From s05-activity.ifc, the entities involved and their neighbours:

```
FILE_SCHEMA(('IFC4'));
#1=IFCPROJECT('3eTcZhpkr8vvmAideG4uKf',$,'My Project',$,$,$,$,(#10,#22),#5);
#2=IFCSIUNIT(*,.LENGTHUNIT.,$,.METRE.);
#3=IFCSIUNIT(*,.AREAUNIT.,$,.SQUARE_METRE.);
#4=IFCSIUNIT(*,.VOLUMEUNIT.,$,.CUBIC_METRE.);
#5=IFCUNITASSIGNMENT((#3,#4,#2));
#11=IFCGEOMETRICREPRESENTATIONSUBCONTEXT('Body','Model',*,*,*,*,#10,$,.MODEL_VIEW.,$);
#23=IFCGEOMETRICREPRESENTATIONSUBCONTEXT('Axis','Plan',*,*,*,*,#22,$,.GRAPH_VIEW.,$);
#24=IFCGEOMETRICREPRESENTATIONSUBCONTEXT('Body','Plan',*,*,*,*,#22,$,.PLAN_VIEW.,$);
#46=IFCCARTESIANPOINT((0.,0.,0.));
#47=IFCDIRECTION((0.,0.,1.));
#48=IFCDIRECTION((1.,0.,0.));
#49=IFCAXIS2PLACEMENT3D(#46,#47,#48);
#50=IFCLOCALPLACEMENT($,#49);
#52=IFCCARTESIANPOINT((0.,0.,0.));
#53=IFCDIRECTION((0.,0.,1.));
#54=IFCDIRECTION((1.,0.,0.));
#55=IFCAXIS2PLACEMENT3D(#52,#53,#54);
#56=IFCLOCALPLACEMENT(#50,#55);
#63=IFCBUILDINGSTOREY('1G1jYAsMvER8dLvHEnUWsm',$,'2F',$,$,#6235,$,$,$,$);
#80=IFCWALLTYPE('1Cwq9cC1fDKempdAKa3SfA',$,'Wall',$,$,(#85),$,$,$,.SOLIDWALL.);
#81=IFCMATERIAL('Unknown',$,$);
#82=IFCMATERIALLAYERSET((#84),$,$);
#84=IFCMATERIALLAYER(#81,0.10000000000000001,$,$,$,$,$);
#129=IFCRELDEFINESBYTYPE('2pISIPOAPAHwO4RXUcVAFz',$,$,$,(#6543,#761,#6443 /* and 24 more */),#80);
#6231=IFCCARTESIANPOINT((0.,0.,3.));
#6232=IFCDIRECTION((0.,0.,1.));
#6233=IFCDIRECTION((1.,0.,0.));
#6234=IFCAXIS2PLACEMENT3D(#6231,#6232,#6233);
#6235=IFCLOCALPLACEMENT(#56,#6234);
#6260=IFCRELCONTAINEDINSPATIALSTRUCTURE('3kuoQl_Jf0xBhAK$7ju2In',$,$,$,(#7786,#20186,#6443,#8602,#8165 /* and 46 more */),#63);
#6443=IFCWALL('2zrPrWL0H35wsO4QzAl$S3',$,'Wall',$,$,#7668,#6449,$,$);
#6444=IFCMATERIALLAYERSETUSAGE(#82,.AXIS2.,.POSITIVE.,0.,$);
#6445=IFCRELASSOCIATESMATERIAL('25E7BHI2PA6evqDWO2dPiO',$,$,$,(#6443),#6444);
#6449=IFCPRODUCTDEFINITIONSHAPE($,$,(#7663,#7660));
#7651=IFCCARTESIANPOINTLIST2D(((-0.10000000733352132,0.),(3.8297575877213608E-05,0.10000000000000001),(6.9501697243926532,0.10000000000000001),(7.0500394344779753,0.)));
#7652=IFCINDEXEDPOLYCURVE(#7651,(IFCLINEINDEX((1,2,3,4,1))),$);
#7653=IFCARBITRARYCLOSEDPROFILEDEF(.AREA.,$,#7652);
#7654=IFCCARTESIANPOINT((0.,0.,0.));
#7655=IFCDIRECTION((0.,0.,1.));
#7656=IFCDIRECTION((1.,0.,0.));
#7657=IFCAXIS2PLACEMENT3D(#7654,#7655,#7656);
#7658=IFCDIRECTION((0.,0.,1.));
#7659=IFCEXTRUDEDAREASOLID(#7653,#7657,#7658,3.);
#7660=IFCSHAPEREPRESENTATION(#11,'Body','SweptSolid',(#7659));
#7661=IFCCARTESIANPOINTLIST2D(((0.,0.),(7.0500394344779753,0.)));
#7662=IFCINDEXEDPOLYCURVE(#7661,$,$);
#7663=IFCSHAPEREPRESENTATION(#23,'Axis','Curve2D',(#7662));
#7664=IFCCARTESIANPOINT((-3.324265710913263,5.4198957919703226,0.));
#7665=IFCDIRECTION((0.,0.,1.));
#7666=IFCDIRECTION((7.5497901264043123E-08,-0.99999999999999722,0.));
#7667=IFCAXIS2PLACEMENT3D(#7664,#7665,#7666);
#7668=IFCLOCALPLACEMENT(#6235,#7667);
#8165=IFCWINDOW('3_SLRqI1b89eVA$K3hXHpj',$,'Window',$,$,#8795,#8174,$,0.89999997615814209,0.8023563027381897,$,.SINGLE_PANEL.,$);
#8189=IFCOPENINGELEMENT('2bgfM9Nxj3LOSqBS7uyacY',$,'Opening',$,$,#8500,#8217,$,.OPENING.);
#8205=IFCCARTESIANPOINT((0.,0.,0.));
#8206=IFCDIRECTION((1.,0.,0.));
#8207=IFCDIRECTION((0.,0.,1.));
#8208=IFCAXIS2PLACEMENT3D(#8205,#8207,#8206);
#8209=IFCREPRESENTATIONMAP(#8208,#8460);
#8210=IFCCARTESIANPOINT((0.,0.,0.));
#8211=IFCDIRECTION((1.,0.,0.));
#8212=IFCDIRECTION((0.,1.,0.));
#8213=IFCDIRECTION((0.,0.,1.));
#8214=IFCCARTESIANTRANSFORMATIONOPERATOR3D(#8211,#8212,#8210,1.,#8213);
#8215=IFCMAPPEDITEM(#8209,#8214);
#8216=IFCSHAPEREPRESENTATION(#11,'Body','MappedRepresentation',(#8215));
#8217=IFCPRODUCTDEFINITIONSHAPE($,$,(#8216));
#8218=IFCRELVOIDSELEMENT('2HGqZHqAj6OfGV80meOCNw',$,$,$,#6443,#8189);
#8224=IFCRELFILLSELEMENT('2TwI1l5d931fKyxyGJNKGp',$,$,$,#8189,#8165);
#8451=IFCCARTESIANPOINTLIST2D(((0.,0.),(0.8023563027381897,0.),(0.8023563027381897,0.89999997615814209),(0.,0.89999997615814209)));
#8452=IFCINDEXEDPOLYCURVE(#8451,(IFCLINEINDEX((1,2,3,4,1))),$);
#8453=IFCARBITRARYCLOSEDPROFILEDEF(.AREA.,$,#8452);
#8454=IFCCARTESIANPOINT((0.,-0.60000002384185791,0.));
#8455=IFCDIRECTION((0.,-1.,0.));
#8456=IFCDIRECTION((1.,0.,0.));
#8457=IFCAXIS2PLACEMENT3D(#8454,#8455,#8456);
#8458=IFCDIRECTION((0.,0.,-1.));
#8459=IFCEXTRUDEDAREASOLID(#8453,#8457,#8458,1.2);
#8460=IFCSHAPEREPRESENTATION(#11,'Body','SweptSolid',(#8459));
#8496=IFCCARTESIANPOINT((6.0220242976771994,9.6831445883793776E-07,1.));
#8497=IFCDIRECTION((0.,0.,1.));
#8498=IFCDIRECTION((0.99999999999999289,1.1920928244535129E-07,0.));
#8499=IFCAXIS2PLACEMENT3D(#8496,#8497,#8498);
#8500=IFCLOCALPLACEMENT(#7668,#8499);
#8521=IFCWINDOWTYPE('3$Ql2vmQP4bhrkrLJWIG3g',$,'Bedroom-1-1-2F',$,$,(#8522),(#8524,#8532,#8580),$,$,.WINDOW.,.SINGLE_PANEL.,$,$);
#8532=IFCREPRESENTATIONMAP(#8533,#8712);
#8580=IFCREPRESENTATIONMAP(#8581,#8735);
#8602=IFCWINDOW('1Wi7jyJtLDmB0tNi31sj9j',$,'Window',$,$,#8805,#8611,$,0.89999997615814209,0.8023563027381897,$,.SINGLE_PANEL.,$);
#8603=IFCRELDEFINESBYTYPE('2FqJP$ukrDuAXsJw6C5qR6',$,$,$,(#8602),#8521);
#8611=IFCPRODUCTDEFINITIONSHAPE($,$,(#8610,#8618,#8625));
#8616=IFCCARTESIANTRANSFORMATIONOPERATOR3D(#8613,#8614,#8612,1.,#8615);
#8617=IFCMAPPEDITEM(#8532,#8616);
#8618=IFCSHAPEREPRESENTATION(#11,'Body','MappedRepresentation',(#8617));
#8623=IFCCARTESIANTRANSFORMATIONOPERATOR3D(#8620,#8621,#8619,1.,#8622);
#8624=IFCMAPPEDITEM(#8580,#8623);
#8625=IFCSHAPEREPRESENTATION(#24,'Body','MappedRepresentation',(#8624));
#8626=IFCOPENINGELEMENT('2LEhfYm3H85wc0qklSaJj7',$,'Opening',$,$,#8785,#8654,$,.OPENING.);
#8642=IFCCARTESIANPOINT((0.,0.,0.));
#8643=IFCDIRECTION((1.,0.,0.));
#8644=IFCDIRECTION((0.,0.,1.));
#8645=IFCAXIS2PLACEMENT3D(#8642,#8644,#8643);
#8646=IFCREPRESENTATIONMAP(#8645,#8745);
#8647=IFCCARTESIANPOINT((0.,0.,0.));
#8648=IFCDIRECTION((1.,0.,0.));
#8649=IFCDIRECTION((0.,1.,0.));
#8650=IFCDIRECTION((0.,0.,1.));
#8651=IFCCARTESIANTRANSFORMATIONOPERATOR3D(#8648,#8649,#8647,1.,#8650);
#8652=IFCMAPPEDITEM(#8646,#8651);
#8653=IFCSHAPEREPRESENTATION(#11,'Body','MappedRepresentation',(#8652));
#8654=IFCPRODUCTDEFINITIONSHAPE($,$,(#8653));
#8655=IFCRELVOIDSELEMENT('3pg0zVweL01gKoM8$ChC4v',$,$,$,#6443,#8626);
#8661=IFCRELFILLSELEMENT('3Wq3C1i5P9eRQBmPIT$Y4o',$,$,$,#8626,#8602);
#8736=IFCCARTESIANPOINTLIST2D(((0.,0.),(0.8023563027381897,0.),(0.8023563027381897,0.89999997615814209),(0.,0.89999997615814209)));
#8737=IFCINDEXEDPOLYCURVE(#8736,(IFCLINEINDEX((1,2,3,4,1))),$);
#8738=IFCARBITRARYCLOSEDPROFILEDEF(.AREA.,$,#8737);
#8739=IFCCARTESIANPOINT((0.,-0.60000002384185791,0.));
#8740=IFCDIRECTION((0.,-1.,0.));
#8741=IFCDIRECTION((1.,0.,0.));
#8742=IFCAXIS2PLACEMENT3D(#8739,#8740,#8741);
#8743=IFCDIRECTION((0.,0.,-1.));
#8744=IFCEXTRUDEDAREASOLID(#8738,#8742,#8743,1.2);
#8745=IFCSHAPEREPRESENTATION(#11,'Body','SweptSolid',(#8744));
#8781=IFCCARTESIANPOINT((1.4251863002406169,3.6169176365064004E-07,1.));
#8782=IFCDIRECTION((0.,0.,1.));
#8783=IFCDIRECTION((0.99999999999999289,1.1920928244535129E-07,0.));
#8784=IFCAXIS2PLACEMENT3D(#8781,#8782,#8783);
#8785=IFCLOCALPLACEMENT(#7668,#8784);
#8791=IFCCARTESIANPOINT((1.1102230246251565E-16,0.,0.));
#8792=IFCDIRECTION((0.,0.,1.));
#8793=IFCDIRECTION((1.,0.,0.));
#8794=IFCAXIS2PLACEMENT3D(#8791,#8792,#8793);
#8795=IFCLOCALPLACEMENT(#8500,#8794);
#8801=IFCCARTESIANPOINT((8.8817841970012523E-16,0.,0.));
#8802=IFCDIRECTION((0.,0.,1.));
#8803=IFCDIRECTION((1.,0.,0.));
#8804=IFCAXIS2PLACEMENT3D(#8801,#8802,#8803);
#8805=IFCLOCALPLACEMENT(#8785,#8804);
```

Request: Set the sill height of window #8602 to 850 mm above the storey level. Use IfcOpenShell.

```python
import numpy as np
import ifcopenshell
import ifcopenshell.api.geometry
import ifcopenshell.geom
import ifcopenshell.util.element
import ifcopenshell.util.placement
import ifcopenshell.util.shape
import ifcopenshell.util.unit

model = ifcopenshell.open("s05-activity.ifc")
unit_scale = ifcopenshell.util.unit.calculate_unit_scale(model)

window = model.by_id(8602)
opening = window.FillsVoids[0].RelatingOpeningElement
storey = ifcopenshell.util.element.get_container(window, ifc_class="IfcBuildingStorey")
level = ifcopenshell.util.placement.get_local_placement(storey.ObjectPlacement)[2, 3]

# The opening's origin need not be at the sill, so measure its lowest point.
shape = ifcopenshell.geom.create_shape(ifcopenshell.geom.settings(), opening)
bottom = ifcopenshell.util.shape.get_shape_bottom_elevation(shape, shape.geometry) / unit_scale
dz = level + 0.85 - bottom

shift = np.array([0.0, 0.0, dz])
# The window is placed relative to its opening, so it follows when the opening moves.
matrix = ifcopenshell.util.placement.get_local_placement(opening.ObjectPlacement)
matrix[:3, 3] += shift
ifcopenshell.api.geometry.edit_object_placement(
    model, product=opening, matrix=matrix, is_si=False, should_transform_children=True
)

print(f"moved by {dz * unit_scale:+.3f} m")

model.write("s05-activity_rev.ifc")
```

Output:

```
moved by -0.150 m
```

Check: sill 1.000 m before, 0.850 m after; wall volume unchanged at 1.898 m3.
